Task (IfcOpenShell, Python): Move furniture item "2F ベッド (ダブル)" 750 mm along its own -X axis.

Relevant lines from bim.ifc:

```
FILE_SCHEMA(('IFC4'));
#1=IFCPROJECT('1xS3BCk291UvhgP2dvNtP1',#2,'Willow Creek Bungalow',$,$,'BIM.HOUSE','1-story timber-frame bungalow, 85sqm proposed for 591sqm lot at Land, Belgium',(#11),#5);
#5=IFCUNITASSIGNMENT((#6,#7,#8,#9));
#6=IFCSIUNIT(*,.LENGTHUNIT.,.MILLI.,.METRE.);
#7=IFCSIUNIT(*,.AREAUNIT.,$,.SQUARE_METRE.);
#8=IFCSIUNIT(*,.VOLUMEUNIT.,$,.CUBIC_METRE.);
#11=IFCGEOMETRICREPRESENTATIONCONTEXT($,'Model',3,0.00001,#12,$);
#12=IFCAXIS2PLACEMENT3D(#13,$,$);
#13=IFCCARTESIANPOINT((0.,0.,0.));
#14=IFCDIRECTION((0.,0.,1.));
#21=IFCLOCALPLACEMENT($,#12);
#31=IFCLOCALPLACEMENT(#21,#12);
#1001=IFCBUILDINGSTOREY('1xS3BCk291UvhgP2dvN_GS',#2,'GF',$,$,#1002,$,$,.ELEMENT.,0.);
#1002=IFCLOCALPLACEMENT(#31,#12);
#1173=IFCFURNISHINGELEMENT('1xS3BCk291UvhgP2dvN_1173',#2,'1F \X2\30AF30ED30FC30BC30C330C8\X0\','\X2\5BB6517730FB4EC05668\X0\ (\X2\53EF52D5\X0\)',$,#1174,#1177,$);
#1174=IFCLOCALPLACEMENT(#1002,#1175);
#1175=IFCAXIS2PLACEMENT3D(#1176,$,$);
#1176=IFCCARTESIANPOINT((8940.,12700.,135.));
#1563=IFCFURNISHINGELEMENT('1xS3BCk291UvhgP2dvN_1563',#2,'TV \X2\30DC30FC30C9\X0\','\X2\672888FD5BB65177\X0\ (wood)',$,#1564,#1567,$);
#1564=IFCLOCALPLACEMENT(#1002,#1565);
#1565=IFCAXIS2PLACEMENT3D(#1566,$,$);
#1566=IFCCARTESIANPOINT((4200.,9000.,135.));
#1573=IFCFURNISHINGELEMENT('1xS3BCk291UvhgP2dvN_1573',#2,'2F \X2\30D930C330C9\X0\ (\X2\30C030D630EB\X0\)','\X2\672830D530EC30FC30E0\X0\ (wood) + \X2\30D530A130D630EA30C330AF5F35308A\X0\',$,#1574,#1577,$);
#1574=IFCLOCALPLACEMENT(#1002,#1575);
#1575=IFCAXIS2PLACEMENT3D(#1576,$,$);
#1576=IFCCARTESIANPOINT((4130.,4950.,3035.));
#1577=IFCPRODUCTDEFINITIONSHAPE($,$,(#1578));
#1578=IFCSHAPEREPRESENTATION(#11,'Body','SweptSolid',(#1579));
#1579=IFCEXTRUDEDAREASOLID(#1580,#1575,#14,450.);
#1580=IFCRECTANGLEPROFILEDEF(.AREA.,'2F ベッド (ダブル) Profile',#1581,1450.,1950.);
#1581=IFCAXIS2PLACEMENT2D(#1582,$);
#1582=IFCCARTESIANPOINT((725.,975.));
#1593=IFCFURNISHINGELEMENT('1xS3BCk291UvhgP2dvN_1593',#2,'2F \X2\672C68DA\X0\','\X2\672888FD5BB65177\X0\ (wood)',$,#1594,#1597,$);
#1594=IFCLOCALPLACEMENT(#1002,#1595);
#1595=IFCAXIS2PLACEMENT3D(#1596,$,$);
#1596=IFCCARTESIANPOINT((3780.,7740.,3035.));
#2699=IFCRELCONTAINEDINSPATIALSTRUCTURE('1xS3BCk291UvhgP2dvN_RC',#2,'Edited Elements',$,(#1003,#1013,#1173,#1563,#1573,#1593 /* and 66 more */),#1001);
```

```python
import ifcopenshell
import ifcopenshell.api.geometry
import ifcopenshell.util.placement

model = ifcopenshell.open("bim.ifc")

item = model.by_id(1573)
matrix = ifcopenshell.util.placement.get_local_placement(item.ObjectPlacement)
matrix[:3, 3] -= matrix[:3, 0] * 750.0
ifcopenshell.api.geometry.edit_object_placement(model, product=item, matrix=matrix, is_si=False)

print(ifcopenshell.util.placement.get_local_placement(item.ObjectPlacement).round(3) + 0.0)

model.write("bim_updated.ifc")
```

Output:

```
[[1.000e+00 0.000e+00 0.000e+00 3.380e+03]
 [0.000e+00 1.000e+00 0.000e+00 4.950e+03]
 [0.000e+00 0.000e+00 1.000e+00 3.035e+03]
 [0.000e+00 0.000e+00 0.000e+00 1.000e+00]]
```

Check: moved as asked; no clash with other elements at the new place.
